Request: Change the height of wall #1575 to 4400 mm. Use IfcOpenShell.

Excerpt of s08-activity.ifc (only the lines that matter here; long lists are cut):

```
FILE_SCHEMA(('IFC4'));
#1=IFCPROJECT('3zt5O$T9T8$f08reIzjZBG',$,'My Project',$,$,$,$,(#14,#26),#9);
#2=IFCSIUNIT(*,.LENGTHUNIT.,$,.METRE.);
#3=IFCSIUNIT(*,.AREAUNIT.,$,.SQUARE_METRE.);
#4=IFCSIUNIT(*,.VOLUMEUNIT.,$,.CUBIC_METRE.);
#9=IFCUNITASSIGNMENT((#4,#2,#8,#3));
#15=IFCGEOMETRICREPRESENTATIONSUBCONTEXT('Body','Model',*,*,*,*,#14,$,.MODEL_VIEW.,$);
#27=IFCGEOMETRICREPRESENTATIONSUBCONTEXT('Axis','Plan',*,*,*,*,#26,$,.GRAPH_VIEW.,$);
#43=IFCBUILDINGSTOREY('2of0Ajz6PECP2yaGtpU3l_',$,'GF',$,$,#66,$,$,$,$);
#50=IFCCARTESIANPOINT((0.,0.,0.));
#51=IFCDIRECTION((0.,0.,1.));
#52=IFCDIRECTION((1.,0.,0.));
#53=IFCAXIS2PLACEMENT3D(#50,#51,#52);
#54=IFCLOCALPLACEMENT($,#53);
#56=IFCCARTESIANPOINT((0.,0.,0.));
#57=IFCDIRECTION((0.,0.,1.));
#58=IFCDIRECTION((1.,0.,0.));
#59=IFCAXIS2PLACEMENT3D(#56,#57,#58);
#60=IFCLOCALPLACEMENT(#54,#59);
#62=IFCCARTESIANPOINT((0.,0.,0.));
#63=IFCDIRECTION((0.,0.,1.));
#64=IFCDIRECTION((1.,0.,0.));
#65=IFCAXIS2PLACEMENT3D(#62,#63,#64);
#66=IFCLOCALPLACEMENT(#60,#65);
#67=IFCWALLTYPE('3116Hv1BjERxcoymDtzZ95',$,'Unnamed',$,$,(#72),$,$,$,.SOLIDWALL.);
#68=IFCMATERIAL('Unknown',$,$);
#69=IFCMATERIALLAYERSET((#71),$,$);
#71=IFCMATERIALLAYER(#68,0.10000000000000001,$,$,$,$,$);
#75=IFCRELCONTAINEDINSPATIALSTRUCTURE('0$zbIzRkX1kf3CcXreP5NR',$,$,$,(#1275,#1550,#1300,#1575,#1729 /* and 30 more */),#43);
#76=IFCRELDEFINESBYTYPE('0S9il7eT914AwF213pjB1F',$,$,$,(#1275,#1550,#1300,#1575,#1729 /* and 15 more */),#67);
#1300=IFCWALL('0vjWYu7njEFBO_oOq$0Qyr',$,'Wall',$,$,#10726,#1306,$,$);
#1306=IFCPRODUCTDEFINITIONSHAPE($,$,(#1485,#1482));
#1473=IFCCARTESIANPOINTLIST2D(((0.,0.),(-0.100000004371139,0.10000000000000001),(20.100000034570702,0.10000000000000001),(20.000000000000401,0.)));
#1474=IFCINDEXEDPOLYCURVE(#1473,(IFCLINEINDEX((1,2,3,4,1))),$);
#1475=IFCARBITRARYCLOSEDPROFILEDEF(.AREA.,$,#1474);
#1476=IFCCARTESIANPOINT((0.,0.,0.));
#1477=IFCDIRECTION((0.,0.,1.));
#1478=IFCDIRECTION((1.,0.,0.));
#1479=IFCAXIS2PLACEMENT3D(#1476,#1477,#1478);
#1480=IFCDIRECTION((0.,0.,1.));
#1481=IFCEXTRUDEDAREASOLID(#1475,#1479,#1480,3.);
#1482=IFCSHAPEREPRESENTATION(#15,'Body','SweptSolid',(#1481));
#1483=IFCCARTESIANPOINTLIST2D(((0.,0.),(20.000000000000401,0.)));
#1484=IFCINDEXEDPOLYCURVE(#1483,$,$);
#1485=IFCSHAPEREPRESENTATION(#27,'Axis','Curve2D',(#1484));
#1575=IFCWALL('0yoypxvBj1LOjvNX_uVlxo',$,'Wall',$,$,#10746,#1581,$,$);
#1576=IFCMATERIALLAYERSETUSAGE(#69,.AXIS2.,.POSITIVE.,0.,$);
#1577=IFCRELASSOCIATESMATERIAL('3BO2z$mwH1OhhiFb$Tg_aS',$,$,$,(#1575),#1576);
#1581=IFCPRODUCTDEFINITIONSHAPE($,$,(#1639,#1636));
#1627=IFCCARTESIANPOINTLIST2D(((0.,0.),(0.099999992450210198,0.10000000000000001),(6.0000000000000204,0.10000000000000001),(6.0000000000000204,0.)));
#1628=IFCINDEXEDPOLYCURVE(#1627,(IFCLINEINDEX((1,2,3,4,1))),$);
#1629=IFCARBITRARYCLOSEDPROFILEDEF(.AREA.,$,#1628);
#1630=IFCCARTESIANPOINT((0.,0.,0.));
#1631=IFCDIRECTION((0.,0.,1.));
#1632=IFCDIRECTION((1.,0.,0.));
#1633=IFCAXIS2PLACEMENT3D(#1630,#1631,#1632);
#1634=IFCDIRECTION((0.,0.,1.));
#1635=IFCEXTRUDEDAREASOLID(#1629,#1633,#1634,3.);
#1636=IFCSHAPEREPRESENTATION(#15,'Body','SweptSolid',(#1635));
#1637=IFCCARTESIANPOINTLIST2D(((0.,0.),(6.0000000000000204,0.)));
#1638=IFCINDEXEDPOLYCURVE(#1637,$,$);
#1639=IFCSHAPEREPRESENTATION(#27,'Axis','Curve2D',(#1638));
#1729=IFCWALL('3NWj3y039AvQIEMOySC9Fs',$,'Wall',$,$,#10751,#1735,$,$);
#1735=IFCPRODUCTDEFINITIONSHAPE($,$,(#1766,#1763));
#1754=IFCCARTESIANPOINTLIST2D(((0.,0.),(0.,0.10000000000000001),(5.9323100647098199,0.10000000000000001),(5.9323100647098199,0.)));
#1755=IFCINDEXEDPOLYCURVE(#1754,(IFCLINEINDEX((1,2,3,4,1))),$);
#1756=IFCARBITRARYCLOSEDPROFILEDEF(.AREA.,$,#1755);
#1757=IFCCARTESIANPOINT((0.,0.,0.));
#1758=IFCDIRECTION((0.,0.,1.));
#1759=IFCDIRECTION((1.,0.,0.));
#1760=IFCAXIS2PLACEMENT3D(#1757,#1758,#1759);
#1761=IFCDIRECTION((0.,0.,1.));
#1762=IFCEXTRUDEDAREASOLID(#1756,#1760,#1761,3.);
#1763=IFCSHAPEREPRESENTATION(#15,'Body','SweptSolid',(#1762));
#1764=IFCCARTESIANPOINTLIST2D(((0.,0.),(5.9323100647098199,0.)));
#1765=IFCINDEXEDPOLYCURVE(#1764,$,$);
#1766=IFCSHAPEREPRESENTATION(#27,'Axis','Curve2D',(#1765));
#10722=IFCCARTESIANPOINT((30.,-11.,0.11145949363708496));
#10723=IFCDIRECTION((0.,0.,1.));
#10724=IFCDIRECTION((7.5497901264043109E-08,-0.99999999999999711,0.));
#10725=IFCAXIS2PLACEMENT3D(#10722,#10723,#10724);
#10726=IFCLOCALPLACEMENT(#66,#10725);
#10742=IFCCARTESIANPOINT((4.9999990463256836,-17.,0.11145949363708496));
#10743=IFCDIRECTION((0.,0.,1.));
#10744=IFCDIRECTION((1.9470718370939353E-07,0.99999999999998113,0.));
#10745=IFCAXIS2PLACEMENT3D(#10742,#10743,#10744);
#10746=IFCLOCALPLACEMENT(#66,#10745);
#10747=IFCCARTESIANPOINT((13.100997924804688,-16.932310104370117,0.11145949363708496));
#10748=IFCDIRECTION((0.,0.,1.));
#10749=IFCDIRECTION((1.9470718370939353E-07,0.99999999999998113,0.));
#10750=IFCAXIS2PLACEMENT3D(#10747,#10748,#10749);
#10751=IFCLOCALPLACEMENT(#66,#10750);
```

```python
import ifcopenshell
import ifcopenshell.geom
import ifcopenshell.util.representation
import ifcopenshell.util.shape

model = ifcopenshell.open("s08-activity.ifc")
settings = ifcopenshell.geom.settings()


def volume(element):
    """Net volume in cubic metres, openings subtracted."""
    shape = ifcopenshell.geom.create_shape(settings, element)
    return ifcopenshell.util.shape.get_volume(shape.geometry)


wall = model.by_id(1575)
before = volume(wall)

body = ifcopenshell.util.representation.get_representation(wall, "Model", "Body")
solid = body.Items[0]
old_height = solid.Depth
solid.Depth = 4.4
after = volume(wall)

print(f"height {old_height:g} -> {solid.Depth:g}, volume {before:.3f} -> {after:.3f} m3")

model.write("s08-activity_v2.ifc")
```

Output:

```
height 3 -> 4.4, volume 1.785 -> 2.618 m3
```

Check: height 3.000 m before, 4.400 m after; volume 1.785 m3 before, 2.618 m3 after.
